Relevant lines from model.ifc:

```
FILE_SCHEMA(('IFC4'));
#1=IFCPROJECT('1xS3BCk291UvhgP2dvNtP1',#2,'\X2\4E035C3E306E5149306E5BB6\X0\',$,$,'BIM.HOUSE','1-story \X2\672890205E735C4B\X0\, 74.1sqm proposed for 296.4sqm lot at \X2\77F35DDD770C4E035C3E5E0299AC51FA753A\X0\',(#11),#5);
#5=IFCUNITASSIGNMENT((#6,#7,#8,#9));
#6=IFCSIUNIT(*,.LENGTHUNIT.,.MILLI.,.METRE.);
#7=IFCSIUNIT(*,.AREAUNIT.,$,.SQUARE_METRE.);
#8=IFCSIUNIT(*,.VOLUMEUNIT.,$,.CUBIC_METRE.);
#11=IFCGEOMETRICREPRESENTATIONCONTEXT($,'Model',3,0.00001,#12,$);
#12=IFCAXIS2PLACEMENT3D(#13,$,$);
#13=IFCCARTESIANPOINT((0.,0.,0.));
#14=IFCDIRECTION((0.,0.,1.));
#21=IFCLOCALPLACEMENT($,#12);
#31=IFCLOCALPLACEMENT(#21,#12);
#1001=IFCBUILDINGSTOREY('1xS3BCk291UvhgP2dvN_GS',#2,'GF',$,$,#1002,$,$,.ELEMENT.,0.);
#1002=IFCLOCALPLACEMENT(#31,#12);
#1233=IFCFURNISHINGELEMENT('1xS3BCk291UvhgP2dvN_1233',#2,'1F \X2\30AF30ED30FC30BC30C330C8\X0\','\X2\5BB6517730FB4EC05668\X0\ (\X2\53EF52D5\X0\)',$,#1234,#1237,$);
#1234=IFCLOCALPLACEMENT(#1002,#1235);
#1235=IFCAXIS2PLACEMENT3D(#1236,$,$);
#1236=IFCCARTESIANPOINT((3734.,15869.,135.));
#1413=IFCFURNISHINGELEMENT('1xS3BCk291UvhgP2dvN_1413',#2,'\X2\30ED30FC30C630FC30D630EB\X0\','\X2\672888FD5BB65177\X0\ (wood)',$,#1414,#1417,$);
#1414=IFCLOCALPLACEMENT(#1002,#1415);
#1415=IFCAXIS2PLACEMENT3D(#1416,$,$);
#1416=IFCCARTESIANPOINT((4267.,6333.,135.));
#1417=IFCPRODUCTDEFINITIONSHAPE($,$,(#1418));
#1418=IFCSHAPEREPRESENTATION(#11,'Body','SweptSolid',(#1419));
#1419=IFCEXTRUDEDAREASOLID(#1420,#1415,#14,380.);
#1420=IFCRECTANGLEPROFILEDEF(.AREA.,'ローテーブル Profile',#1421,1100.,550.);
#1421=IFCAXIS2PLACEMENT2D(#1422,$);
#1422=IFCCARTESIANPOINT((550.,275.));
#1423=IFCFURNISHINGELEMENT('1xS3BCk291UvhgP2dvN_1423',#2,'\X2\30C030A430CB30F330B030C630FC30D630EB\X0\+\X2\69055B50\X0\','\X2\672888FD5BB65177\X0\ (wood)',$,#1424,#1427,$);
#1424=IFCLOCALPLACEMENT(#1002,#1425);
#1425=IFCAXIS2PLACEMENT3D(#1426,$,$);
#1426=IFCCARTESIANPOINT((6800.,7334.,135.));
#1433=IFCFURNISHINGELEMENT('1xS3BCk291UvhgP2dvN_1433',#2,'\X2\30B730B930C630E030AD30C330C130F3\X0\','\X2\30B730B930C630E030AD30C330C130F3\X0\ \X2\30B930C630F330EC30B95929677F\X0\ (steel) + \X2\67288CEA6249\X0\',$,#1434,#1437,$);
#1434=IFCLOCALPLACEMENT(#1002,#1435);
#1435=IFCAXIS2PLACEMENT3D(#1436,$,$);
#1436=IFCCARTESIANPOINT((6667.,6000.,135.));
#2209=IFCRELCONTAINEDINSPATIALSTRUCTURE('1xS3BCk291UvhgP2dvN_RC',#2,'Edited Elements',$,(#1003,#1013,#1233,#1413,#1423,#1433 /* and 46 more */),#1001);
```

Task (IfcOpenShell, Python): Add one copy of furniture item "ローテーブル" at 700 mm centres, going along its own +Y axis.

```python
import ifcopenshell
import ifcopenshell.api.geometry
import ifcopenshell.api.root
import ifcopenshell.util.element
import ifcopenshell.util.placement

model = ifcopenshell.open("model.ifc")


def reuse_history(source, copy):
    """copy_class also copies each property set's owner history, people and application; keep the originals."""
    for rel in copy.IsDefinedBy:
        if rel.is_a("IfcRelDefinesByProperties") and (history := rel.RelatingPropertyDefinition.OwnerHistory):
            rel.RelatingPropertyDefinition.OwnerHistory = source.OwnerHistory
            ifcopenshell.util.element.remove_deep2(model, history)


source = model.by_id(1413)
base = ifcopenshell.util.placement.get_local_placement(source.ObjectPlacement)
step = base[:3, 1] * 700.0

for i in range(1, 2):
    copy = ifcopenshell.api.root.copy_class(model, product=source)
    copy.Representation = ifcopenshell.util.element.copy_deep(
        model, source.Representation, exclude=["IfcGeometricRepresentationContext", "IfcRepresentationMap"]
    )
    reuse_history(source, copy)
    matrix = base.copy()
    matrix[:3, 3] += i * step
    print("added at", matrix[:3, 3].round(3) + 0.0)
    ifcopenshell.api.geometry.edit_object_placement(model, product=copy, matrix=matrix, is_si=False)

model.write("model_edited.ifc")
```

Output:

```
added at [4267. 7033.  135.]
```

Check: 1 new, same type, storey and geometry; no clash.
